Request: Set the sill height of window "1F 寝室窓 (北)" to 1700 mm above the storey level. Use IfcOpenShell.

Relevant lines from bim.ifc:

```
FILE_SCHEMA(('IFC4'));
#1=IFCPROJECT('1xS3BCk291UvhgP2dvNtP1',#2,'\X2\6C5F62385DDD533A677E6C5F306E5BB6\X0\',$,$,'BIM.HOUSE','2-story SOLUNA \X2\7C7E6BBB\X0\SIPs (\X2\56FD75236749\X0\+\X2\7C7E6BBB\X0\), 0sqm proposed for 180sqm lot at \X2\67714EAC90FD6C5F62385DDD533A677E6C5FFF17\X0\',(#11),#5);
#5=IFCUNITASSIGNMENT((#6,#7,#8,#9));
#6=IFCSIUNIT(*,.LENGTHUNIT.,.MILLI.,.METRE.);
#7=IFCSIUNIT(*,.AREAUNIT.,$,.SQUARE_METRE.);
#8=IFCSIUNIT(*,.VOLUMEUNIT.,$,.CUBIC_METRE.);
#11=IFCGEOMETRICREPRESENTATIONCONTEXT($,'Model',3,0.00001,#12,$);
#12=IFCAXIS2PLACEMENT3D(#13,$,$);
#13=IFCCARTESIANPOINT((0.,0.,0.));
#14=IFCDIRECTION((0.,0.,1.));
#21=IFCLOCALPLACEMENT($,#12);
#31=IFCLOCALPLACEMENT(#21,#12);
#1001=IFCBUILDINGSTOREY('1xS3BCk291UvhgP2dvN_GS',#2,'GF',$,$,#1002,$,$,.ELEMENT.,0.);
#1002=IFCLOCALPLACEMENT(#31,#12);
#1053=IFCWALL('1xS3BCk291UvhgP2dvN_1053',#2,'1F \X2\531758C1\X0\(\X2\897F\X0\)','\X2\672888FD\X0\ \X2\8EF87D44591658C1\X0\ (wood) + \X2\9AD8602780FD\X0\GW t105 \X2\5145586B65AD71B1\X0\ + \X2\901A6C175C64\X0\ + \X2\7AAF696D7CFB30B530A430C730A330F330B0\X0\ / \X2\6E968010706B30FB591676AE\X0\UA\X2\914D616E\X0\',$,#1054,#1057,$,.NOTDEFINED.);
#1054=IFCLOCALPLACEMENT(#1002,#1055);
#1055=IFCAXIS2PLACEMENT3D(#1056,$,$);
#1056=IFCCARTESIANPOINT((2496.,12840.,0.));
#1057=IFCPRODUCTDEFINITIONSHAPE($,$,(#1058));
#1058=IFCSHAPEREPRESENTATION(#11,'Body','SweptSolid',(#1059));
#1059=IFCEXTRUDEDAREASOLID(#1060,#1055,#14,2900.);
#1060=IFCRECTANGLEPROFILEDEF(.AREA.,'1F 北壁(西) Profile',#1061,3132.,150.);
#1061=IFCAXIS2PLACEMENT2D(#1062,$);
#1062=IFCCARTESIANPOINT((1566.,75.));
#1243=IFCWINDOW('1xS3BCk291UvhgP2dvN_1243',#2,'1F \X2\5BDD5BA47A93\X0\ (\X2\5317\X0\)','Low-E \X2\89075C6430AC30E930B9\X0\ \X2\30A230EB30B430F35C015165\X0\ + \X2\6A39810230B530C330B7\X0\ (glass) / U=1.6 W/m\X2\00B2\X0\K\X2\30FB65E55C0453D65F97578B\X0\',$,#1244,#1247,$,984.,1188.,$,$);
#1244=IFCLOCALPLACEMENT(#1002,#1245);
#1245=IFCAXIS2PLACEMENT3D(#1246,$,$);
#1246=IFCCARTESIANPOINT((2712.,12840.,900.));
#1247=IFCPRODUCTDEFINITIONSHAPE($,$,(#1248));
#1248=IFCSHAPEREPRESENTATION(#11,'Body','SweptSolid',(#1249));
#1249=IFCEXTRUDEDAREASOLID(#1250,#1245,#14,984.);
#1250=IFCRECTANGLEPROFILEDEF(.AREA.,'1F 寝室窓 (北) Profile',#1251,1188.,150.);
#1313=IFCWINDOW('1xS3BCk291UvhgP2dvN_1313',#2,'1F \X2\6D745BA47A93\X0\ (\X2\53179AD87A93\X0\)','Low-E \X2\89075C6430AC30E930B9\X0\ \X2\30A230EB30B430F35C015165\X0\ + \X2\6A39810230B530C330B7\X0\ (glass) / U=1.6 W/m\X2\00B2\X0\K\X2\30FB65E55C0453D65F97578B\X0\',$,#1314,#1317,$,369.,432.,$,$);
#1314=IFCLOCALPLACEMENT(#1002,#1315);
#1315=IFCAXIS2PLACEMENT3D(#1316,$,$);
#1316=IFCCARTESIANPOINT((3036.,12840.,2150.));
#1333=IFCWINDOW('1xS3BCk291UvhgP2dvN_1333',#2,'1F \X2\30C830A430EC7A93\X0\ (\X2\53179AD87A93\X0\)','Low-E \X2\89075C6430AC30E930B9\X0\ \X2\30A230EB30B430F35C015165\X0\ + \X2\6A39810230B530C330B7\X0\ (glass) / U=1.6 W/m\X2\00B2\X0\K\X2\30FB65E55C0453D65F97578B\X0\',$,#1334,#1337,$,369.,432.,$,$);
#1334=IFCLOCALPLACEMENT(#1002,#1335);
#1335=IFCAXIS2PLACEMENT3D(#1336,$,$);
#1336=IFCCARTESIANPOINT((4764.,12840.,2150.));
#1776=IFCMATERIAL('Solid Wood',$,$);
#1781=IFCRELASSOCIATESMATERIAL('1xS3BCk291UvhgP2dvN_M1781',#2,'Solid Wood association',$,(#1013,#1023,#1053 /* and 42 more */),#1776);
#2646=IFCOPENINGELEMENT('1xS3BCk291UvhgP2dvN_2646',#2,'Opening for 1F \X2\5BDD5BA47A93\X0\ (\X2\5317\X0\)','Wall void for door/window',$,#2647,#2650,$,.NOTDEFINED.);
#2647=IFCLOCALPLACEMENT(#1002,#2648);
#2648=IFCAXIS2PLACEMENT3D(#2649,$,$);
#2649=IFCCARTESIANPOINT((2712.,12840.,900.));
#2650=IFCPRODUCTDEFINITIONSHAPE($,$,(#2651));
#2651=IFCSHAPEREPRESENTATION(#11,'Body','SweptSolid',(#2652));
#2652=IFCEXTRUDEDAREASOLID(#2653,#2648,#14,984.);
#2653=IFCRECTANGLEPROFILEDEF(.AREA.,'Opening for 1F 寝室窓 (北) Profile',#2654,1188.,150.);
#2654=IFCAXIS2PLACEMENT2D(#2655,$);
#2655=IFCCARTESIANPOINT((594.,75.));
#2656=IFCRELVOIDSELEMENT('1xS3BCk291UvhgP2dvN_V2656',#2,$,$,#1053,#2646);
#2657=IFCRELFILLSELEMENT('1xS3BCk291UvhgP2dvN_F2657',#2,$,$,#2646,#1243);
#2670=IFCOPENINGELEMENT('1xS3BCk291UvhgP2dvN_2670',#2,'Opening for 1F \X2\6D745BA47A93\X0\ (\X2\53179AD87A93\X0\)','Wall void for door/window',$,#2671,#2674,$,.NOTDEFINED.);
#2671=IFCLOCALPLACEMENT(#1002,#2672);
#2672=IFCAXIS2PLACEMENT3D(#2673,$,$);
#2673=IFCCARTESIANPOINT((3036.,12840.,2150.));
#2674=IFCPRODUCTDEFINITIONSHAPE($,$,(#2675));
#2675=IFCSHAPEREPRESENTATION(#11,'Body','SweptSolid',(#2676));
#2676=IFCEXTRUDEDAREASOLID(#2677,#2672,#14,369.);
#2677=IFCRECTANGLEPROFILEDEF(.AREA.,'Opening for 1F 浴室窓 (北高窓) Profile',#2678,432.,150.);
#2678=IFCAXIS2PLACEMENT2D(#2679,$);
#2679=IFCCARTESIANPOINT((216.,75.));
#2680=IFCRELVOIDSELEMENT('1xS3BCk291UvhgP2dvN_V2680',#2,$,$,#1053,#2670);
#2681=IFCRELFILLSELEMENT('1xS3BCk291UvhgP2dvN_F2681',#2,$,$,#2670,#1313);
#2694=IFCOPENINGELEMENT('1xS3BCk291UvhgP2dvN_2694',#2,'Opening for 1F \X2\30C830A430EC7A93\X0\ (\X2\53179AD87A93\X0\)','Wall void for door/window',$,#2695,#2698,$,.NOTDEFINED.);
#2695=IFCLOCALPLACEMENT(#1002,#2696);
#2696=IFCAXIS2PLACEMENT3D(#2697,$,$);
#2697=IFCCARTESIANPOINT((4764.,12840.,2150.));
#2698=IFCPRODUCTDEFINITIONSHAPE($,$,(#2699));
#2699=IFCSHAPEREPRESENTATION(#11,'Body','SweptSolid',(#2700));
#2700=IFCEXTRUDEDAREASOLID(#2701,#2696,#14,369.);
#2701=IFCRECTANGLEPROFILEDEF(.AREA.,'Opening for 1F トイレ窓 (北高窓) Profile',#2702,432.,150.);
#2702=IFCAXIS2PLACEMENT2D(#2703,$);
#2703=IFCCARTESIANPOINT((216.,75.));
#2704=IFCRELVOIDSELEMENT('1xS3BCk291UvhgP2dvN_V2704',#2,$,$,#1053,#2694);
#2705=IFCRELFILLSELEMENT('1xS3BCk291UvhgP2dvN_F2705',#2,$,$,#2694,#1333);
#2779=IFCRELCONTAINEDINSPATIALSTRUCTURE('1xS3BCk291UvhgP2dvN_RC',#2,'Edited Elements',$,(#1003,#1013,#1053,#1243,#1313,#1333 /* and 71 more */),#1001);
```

```python
import numpy as np
import ifcopenshell
import ifcopenshell.api.geometry
import ifcopenshell.geom
import ifcopenshell.util.element
import ifcopenshell.util.placement
import ifcopenshell.util.shape
import ifcopenshell.util.unit

model = ifcopenshell.open("bim.ifc")
unit_scale = ifcopenshell.util.unit.calculate_unit_scale(model)

window = model.by_guid("1xS3BCk291UvhgP2dvN_1243")
opening = window.FillsVoids[0].RelatingOpeningElement
storey = ifcopenshell.util.element.get_container(window, ifc_class="IfcBuildingStorey")
level = ifcopenshell.util.placement.get_local_placement(storey.ObjectPlacement)[2, 3]

# The opening's origin need not be at the sill, so measure its lowest point.
shape = ifcopenshell.geom.create_shape(ifcopenshell.geom.settings(), opening)
bottom = ifcopenshell.util.shape.get_shape_bottom_elevation(shape, shape.geometry) / unit_scale
dz = level + 1.7 / unit_scale - bottom

shift = np.array([0.0, 0.0, dz])
# The window is not placed relative to its opening, so move both.
for product in (opening, window):
    matrix = ifcopenshell.util.placement.get_local_placement(product.ObjectPlacement)
    matrix[:3, 3] += shift
    ifcopenshell.api.geometry.edit_object_placement(model, product=product, matrix=matrix, is_si=False)

print(f"moved by {dz * unit_scale:+.3f} m")

model.write("bim_v2.ifc")
```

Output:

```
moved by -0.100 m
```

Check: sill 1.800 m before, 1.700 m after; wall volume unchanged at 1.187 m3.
